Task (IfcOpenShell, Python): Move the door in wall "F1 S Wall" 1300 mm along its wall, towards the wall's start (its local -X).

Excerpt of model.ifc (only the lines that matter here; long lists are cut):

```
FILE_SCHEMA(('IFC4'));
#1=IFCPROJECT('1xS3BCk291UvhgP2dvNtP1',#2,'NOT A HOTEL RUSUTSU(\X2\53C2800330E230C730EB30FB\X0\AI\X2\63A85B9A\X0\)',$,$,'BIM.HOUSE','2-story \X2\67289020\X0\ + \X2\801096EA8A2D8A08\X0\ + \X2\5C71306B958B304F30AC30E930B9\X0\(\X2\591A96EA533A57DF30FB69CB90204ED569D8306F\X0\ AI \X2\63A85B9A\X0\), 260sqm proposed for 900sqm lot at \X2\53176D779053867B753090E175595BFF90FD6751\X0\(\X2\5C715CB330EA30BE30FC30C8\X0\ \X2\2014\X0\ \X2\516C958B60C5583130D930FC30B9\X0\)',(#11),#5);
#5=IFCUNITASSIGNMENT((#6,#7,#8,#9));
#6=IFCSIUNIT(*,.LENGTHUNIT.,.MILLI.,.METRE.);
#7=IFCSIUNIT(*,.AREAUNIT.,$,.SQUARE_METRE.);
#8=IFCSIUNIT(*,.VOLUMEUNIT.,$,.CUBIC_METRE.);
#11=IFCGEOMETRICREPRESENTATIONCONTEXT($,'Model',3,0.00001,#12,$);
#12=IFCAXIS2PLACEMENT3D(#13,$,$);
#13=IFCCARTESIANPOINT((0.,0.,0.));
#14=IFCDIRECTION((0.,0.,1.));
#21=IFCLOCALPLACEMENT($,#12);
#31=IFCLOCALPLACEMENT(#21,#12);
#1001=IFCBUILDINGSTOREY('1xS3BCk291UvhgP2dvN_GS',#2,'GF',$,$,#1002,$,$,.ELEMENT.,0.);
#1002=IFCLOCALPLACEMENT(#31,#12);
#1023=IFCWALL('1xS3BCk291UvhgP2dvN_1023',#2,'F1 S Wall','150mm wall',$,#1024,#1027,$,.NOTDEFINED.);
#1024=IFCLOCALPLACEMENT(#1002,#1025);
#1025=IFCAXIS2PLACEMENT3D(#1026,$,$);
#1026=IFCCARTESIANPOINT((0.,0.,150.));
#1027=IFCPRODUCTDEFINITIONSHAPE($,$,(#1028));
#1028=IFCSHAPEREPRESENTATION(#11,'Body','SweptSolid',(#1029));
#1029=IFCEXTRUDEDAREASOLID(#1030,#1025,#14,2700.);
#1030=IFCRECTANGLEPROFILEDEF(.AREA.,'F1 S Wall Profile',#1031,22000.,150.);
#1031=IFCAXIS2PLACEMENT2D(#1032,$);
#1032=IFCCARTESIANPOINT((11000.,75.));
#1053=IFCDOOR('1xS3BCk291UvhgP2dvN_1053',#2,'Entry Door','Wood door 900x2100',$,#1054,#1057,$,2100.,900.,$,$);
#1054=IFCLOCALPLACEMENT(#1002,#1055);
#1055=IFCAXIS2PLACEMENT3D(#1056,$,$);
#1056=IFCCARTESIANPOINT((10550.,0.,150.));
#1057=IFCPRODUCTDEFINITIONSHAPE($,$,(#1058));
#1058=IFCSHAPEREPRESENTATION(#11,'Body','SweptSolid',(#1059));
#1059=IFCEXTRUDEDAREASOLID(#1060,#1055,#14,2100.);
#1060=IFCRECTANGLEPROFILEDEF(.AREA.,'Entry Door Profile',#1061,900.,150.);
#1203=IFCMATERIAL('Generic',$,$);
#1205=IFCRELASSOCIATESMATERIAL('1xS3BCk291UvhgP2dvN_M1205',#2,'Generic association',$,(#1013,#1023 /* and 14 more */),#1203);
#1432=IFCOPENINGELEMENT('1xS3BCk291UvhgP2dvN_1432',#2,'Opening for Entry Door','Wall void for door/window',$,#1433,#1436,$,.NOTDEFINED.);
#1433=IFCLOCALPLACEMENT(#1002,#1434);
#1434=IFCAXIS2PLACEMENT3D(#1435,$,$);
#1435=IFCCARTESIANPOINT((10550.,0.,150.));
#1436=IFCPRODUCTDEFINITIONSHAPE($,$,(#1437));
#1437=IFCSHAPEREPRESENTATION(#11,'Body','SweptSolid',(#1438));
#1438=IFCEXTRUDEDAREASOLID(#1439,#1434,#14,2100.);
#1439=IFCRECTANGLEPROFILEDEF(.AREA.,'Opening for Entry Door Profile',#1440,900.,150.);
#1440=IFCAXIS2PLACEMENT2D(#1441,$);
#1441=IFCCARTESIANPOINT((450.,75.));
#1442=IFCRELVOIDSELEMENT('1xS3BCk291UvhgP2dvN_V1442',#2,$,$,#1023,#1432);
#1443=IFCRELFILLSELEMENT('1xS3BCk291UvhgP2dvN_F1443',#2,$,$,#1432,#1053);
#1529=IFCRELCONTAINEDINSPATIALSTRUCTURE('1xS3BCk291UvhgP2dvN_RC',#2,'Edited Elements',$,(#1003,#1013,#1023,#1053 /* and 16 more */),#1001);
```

```python
import ifcopenshell
import ifcopenshell.api.geometry
import ifcopenshell.util.placement

model = ifcopenshell.open("model.ifc")

door = model.by_guid("1xS3BCk291UvhgP2dvN_1053")
opening = door.FillsVoids[0].RelatingOpeningElement
wall = opening.VoidsElements[0].RelatingBuildingElement

wall_matrix = ifcopenshell.util.placement.get_local_placement(wall.ObjectPlacement)
shift = wall_matrix[:3, 0] * -1300.0
before = ifcopenshell.util.placement.get_local_placement(door.ObjectPlacement)[:3, 3].copy()

# The door is not placed relative to its opening, so move both.
for product in (opening, door):
    matrix = ifcopenshell.util.placement.get_local_placement(product.ObjectPlacement)
    matrix[:3, 3] += shift
    ifcopenshell.api.geometry.edit_object_placement(model, product=product, matrix=matrix, is_si=False)

after = ifcopenshell.util.placement.get_local_placement(door.ObjectPlacement)[:3, 3]
print("door moved by", (after - before).round(3) + 0.0)

model.write("model_edited.ifc")
```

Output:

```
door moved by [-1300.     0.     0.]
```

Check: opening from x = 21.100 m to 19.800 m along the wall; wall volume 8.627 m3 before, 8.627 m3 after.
